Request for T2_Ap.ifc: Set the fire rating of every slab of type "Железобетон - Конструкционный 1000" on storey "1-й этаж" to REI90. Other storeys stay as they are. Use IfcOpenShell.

First a look at what the model holds.

```python
import ifcopenshell
import ifcopenshell.util.element

model = ifcopenshell.open("T2_Ap.ifc")
print(model.schema)
storey = next(s for s in model.by_type("IfcBuildingStorey") if s.Name == "1-й этаж")
slabs = [e for e in ifcopenshell.util.element.get_decomposition(storey) if e.is_a("IfcSlab")]
seen = {}
for e in slabs:
    element_type = ifcopenshell.util.element.get_type(e)
    key = (element_type.Name if element_type != e and element_type else None, ifcopenshell.util.element.get_pset(e, "Pset_SlabCommon", "FireRating"))
    seen[key] = seen.get(key, 0) + 1
for (name, value), count in sorted(seen.items(), key=str):
    print(count, "x", name, "|", value)
```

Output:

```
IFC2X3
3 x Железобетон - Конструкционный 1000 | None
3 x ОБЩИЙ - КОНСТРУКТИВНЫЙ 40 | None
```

```python
import ifcopenshell
import ifcopenshell.api.pset
import ifcopenshell.util.element

model = ifcopenshell.open("T2_Ap.ifc")

storey = next(s for s in model.by_type("IfcBuildingStorey") if s.Name == "1-й этаж")
slabs = [e for e in ifcopenshell.util.element.get_decomposition(storey) if e.is_a("IfcSlab")]

count = 0
for e in slabs:
    element_type = ifcopenshell.util.element.get_type(e)
    if element_type in (None, e) or element_type.Name != "Железобетон - Конструкционный 1000":
        continue
    # add_pset returns the element's existing set when there is one.
    pset = ifcopenshell.api.pset.add_pset(model, product=e, name="Pset_SlabCommon")
    ifcopenshell.api.pset.edit_pset(model, pset=pset, properties={"FireRating": "REI90"})
    count += 1

print(count, "slabs updated")

model.write("T2_Ap_edited.ifc")
```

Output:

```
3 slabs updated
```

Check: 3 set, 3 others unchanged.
